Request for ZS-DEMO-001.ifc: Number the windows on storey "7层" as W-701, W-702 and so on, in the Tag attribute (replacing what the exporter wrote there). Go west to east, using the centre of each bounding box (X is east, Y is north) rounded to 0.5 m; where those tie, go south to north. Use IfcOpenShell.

First a look at what the model holds.

```python
import ifcopenshell
import ifcopenshell.util.element
import ifcopenshell.util.placement

model = ifcopenshell.open("ZS-DEMO-001.ifc")
print(model.schema)
storey = next(s for s in model.by_type("IfcBuildingStorey") if s.Name == "7层")
windows = [e for e in ifcopenshell.util.element.get_decomposition(storey) if e.is_a("IfcWindow")]
for e in sorted(windows, key=lambda e: e.id()):
    origin = ifcopenshell.util.placement.get_local_placement(e.ObjectPlacement)[:3, 3]
    print(e.id(), e.Tag, e.Name, origin.round(2) + 0.0, sep=" | ")
```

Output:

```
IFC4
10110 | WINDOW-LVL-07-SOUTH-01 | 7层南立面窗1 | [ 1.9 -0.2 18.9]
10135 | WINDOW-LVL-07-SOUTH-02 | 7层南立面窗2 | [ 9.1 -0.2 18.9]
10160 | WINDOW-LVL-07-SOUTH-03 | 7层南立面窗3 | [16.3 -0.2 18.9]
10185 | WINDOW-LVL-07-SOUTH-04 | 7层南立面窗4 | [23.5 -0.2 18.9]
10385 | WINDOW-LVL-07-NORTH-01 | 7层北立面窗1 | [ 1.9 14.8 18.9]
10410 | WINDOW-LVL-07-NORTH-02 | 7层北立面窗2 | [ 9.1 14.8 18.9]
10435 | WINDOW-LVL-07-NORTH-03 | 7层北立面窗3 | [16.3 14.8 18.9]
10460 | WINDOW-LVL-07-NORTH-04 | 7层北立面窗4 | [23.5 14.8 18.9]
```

```python
import ifcopenshell
import ifcopenshell.geom
import ifcopenshell.util.element
import ifcopenshell.util.shape

model = ifcopenshell.open("ZS-DEMO-001.ifc")
settings = ifcopenshell.geom.settings()
settings.set("use-world-coords", True)


def centre(element):
    shape = ifcopenshell.geom.create_shape(settings, element)
    return ifcopenshell.util.shape.get_bbox_centroid(shape.geometry)


storey = next(s for s in model.by_type("IfcBuildingStorey") if s.Name == "7层")
windows = [e for e in ifcopenshell.util.element.get_decomposition(storey) if e.is_a("IfcWindow")]

# Insertion points can sit at a corner or the storey origin, so sort by the geometry (in metres).
centres = {e: centre(e) for e in windows}
windows.sort(key=lambda e: (round(centres[e][0] / 0.5), centres[e][1]))

for i, e in enumerate(windows, start=1):
    number = f"W-7{i:02d}"
    e.Tag = number
    print(e.id(), number)

model.write("ZS-DEMO-001_v2.ifc")
```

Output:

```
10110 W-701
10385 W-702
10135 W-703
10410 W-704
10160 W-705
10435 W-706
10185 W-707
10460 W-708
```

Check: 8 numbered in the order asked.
